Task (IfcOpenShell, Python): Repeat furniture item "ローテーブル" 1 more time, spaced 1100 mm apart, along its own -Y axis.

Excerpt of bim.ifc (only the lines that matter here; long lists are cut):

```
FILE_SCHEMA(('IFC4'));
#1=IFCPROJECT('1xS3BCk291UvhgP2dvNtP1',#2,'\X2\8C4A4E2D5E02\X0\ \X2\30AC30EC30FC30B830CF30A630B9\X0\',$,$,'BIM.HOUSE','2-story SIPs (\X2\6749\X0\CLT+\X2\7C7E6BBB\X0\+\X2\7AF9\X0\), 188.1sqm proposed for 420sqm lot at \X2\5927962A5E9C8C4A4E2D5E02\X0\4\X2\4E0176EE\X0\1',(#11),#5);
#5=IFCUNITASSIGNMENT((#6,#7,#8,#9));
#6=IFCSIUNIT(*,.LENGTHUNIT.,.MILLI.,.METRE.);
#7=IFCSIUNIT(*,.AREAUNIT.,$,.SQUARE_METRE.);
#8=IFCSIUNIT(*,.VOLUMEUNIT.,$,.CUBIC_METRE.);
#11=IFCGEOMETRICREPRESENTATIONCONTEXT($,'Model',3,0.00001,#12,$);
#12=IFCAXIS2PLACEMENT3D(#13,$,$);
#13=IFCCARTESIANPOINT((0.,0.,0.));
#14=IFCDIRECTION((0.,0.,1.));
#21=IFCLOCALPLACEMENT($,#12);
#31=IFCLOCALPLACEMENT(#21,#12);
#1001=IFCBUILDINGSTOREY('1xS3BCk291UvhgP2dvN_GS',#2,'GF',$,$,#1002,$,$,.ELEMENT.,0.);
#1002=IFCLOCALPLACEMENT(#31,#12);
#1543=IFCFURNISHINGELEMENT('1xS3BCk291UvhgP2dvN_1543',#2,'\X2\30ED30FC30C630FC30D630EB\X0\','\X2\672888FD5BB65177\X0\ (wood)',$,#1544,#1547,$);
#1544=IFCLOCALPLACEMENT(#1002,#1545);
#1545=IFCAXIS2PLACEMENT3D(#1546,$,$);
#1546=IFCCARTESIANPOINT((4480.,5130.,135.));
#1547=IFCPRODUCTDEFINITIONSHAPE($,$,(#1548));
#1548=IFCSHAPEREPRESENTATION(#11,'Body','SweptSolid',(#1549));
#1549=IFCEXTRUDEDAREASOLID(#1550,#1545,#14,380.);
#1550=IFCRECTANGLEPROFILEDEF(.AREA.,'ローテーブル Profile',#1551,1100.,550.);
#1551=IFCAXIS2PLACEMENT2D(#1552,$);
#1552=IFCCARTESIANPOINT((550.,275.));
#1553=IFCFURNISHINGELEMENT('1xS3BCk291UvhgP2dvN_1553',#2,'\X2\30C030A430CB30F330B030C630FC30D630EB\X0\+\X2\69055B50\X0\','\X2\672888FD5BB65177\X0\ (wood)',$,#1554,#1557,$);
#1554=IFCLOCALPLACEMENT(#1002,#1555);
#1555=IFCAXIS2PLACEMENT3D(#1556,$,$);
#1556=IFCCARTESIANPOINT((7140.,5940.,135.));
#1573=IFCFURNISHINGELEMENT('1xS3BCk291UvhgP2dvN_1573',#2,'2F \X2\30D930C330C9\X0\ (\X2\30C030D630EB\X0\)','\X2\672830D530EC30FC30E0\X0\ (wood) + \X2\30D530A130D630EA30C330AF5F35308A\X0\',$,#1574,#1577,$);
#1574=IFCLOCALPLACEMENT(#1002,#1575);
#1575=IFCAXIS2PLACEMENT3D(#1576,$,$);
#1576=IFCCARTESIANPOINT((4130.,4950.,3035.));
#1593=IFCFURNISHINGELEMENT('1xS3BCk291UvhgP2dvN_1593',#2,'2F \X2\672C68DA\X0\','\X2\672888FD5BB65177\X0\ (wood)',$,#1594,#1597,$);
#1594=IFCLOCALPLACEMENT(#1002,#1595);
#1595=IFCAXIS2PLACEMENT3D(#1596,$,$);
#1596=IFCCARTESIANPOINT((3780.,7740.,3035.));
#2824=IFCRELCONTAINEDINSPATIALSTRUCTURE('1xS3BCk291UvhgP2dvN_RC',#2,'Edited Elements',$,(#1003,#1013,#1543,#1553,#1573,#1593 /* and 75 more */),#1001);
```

```python
import ifcopenshell
import ifcopenshell.api.geometry
import ifcopenshell.api.root
import ifcopenshell.util.element
import ifcopenshell.util.placement

model = ifcopenshell.open("bim.ifc")


def reuse_history(source, copy):
    """copy_class also copies each property set's owner history, people and application; keep the originals."""
    for rel in copy.IsDefinedBy:
        if rel.is_a("IfcRelDefinesByProperties") and (history := rel.RelatingPropertyDefinition.OwnerHistory):
            rel.RelatingPropertyDefinition.OwnerHistory = source.OwnerHistory
            ifcopenshell.util.element.remove_deep2(model, history)


source = model.by_guid("1xS3BCk291UvhgP2dvN_1543")
base = ifcopenshell.util.placement.get_local_placement(source.ObjectPlacement)
step = -base[:3, 1] * 1100.0

for i in range(1, 2):
    copy = ifcopenshell.api.root.copy_class(model, product=source)
    copy.Representation = ifcopenshell.util.element.copy_deep(
        model, source.Representation, exclude=["IfcGeometricRepresentationContext", "IfcRepresentationMap"]
    )
    reuse_history(source, copy)
    matrix = base.copy()
    matrix[:3, 3] += i * step
    print("added at", matrix[:3, 3].round(3) + 0.0)
    ifcopenshell.api.geometry.edit_object_placement(model, product=copy, matrix=matrix, is_si=False)

model.write("bim_updated.ifc")
```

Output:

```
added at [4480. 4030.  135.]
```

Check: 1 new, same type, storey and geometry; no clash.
